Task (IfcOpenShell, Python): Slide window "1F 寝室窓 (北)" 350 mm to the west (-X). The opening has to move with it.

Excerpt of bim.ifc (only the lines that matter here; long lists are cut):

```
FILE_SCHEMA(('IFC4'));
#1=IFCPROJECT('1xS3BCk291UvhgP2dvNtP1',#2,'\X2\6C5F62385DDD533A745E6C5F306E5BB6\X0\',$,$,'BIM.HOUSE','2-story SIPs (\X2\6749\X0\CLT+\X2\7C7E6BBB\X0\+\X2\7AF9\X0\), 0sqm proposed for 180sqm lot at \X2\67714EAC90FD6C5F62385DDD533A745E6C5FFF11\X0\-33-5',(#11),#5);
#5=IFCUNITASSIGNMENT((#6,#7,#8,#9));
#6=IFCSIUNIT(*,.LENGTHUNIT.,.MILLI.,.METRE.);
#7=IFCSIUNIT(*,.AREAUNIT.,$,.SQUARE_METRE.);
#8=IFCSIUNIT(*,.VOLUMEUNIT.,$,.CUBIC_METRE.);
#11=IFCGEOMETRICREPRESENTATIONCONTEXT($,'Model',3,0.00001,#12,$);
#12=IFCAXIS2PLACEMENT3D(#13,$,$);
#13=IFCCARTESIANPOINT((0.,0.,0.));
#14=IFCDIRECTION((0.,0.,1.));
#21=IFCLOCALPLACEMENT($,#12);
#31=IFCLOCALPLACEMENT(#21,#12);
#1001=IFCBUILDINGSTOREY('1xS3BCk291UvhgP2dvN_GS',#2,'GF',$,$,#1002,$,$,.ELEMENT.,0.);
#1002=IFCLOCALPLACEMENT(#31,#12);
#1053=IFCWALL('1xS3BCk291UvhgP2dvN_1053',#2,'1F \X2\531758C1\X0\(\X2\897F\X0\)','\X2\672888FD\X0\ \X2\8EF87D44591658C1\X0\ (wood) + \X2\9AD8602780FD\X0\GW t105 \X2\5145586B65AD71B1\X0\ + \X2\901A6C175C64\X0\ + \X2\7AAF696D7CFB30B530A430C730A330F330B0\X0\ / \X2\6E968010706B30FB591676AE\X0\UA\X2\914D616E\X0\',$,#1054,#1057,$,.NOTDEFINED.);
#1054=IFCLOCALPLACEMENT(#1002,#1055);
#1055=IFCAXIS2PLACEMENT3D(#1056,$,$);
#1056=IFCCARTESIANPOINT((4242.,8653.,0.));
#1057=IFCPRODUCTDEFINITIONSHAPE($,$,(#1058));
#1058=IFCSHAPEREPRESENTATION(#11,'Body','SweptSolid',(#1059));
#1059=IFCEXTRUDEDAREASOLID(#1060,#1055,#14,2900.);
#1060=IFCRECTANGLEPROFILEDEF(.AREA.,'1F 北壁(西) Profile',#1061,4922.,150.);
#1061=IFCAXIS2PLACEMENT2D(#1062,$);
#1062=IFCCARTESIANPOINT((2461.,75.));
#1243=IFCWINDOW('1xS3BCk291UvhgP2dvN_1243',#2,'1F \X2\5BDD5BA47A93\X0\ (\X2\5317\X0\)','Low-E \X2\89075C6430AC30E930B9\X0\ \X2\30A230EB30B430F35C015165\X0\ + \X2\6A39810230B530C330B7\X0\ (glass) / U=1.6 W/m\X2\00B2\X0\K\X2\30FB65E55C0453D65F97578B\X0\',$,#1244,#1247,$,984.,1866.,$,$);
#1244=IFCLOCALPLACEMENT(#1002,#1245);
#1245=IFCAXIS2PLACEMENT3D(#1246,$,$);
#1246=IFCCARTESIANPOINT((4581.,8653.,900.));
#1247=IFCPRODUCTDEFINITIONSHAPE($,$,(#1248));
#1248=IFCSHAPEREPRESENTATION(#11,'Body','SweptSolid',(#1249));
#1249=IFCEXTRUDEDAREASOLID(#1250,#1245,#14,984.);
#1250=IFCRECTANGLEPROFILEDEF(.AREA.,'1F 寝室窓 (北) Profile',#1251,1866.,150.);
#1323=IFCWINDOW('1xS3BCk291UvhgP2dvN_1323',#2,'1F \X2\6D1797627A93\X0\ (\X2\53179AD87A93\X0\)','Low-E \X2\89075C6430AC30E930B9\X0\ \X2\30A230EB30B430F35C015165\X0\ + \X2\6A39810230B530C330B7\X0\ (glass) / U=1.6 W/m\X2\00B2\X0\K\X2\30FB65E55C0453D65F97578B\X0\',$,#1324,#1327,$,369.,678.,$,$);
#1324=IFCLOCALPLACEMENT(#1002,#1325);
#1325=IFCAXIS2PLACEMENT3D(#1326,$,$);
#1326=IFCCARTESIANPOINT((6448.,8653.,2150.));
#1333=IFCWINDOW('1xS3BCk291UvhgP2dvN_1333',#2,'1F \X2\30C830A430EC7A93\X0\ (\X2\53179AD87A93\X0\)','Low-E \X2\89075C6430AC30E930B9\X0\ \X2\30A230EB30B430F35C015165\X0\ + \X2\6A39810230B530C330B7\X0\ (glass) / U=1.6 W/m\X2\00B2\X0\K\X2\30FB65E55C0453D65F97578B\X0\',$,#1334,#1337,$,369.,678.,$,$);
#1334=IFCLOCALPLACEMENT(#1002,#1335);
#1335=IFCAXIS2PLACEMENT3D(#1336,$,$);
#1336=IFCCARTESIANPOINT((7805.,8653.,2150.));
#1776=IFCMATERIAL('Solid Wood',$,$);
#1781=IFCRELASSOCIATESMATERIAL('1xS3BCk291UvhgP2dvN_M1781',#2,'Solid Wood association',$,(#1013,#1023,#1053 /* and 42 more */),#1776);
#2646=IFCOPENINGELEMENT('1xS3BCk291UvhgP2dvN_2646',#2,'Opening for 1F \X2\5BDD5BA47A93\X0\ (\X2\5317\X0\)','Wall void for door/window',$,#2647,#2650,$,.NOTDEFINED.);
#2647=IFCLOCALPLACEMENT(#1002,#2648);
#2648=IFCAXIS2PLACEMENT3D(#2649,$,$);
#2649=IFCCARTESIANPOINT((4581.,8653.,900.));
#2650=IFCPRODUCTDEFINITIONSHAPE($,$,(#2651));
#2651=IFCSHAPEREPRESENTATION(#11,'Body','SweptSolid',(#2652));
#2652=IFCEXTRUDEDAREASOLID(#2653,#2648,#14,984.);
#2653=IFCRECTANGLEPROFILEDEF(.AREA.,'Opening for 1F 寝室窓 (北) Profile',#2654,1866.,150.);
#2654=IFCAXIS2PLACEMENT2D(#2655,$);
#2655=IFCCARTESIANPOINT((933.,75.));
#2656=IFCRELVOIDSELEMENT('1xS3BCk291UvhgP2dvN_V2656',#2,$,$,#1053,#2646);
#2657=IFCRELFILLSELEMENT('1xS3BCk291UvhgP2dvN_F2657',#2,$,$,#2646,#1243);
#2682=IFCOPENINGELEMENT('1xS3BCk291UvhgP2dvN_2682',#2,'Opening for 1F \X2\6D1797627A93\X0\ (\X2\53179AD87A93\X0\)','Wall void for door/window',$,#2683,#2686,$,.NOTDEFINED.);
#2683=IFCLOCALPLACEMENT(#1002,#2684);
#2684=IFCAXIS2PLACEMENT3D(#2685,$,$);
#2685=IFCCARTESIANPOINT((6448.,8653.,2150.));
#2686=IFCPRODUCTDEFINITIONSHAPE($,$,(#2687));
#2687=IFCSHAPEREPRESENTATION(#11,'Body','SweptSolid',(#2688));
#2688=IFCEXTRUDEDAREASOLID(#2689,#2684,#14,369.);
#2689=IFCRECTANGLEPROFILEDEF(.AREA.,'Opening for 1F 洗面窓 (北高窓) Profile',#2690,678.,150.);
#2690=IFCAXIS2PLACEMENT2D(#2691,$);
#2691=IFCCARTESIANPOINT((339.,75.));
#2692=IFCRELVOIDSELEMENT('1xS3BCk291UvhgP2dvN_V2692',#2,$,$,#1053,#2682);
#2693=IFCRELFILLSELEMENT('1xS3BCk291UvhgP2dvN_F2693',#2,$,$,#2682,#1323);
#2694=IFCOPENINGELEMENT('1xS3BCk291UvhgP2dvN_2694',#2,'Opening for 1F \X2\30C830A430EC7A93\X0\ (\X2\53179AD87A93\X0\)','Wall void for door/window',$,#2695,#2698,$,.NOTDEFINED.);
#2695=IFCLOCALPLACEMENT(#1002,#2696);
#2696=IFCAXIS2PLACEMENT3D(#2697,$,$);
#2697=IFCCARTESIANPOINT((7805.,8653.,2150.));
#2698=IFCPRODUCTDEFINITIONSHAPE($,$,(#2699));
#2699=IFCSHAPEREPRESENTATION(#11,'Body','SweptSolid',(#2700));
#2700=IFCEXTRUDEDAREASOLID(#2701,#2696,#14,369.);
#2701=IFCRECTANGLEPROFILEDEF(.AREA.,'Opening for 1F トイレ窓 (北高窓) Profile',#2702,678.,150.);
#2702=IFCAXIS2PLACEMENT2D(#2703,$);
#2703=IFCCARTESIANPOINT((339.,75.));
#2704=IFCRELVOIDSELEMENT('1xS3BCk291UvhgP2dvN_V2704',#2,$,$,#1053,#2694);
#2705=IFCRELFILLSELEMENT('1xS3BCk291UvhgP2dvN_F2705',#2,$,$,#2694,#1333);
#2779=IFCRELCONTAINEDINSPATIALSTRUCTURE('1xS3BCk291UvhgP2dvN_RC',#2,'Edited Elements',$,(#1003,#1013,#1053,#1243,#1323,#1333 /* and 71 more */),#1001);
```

```python
import ifcopenshell
import ifcopenshell.api.geometry
import ifcopenshell.util.placement

model = ifcopenshell.open("bim.ifc")

window = model.by_id(1243)
opening = window.FillsVoids[0].RelatingOpeningElement
wall = opening.VoidsElements[0].RelatingBuildingElement

wall_matrix = ifcopenshell.util.placement.get_local_placement(wall.ObjectPlacement)
shift = wall_matrix[:3, 0] * -350.0
before = ifcopenshell.util.placement.get_local_placement(window.ObjectPlacement)[:3, 3].copy()

# The window is not placed relative to its opening, so move both.
for product in (opening, window):
    matrix = ifcopenshell.util.placement.get_local_placement(product.ObjectPlacement)
    matrix[:3, 3] += shift
    ifcopenshell.api.geometry.edit_object_placement(model, product=product, matrix=matrix, is_si=False)

after = ifcopenshell.util.placement.get_local_placement(window.ObjectPlacement)[:3, 3]
print("window moved by", (after - before).round(3) + 0.0)

model.write("bim_v2.ifc")
```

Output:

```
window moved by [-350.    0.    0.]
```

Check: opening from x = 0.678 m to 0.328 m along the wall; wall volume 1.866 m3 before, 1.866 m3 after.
